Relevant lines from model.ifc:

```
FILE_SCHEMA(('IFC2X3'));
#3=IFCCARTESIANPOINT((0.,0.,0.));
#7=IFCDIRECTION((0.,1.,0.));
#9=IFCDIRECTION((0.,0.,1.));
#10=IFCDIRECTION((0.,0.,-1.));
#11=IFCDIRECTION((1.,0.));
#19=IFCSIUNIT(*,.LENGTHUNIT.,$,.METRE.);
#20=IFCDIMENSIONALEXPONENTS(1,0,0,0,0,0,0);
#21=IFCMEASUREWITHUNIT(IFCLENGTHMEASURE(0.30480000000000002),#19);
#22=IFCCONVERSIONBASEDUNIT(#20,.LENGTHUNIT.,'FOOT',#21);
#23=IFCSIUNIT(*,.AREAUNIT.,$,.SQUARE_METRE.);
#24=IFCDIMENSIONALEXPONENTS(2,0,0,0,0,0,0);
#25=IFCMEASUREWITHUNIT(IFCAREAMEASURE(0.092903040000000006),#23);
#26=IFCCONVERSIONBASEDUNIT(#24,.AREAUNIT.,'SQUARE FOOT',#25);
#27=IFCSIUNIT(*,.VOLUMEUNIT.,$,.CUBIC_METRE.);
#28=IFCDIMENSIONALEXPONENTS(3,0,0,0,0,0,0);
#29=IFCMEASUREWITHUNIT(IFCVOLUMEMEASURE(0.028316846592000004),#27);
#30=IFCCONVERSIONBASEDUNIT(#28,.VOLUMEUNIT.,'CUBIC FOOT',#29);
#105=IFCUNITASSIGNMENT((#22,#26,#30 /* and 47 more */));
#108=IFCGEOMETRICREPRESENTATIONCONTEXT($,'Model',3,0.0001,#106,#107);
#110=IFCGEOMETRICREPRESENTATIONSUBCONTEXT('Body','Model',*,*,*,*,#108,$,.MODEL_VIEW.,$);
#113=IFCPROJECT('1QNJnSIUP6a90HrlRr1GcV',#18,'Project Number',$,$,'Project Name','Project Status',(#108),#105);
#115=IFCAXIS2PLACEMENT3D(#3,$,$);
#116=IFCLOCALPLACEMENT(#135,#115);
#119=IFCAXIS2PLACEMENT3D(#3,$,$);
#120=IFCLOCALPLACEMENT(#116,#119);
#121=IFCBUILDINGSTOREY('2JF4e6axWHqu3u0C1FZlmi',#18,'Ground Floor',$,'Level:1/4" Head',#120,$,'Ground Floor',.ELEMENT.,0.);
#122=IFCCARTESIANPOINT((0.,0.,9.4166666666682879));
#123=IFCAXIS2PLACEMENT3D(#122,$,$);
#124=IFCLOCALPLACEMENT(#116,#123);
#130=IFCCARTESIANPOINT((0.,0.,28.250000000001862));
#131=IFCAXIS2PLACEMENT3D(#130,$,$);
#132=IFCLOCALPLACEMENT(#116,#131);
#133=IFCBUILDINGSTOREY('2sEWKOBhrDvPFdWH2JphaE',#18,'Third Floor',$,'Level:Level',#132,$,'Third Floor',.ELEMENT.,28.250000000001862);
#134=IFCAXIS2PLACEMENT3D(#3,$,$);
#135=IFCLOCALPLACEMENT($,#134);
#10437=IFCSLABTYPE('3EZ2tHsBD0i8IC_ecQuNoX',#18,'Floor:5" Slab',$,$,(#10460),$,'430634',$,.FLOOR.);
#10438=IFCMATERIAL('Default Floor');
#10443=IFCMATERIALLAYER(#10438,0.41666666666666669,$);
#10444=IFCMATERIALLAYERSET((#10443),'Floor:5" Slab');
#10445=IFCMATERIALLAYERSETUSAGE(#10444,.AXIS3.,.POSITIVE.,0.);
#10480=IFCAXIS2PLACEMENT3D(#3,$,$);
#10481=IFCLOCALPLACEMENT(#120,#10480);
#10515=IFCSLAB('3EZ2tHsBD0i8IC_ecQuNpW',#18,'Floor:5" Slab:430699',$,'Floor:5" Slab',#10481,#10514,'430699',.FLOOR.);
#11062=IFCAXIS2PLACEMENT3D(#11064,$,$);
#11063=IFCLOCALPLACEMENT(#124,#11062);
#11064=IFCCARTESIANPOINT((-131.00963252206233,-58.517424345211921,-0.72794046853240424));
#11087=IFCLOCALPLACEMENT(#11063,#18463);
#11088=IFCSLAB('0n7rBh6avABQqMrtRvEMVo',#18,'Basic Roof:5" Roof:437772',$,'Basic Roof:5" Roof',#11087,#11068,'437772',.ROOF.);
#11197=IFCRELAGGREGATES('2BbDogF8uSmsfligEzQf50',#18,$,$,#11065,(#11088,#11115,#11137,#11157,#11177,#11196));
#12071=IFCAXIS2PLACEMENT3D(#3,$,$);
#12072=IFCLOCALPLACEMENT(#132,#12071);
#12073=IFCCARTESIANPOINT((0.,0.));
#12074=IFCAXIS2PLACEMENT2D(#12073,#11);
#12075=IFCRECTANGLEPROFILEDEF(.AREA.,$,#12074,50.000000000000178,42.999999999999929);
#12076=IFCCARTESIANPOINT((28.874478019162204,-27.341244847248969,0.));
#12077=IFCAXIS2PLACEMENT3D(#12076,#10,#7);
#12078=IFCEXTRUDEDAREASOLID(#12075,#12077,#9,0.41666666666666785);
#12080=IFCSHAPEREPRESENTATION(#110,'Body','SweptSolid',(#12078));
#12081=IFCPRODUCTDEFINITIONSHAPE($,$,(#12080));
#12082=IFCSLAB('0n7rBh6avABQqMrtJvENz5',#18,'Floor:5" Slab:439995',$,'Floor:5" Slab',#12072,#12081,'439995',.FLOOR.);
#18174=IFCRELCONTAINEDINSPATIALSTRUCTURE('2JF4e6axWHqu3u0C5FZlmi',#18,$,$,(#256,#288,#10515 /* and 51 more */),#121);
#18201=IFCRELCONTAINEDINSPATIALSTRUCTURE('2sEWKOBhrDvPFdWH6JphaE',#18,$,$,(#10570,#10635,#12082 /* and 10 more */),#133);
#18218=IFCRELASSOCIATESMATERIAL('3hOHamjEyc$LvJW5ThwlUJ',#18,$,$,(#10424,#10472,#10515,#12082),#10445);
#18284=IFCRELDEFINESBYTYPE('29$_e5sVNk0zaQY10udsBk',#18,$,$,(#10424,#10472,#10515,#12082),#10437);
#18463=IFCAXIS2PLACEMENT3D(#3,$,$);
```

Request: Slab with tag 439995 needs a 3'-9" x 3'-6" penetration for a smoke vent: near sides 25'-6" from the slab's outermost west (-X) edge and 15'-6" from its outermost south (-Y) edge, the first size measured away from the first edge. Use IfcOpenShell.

```python
import numpy as np
import ifcopenshell
import ifcopenshell.api.feature
import ifcopenshell.api.geometry
import ifcopenshell.api.root
import ifcopenshell.geom
import ifcopenshell.util.placement
import ifcopenshell.util.representation
import ifcopenshell.util.shape
import ifcopenshell.util.unit

model = ifcopenshell.open("model.ifc")
unit_scale = ifcopenshell.util.unit.calculate_unit_scale(model)
settings = ifcopenshell.geom.settings()


def volume(element):
    """Net volume in cubic metres, openings subtracted."""
    shape = ifcopenshell.geom.create_shape(settings, element)
    return ifcopenshell.util.shape.get_volume(shape.geometry)


slab = model.by_guid("0n7rBh6avABQqMrtJvENz5")
before = volume(slab)

# Extent in the slab's own axes, in metres. The edges named are its -X and -Y sides.
slab_shape = ifcopenshell.geom.create_shape(settings, slab)
vertices = ifcopenshell.util.shape.get_vertices(slab_shape.geometry)
x_min, y_min, bottom = vertices.min(axis=0)
top = vertices[:, 2].max()

opening = ifcopenshell.api.root.create_entity(model, ifc_class="IfcOpeningElement", name="Smoke vent opening")
context = ifcopenshell.util.representation.get_context(model, "Model", "Body", "MODEL_VIEW")
width, depth = 1.143, 1.0668
outline = [(0.0, 0.0), (width, 0.0), (width, depth), (0.0, depth), (0.0, 0.0)]
# Overshoot both faces by 50 mm so the cut is clean.
shape = ifcopenshell.api.geometry.add_slab_representation(
    model, context=context, depth=top - bottom + 0.1, polyline=outline
)
ifcopenshell.api.geometry.assign_representation(model, product=opening, representation=shape)

matrix = ifcopenshell.util.placement.get_local_placement(slab.ObjectPlacement)
matrix[:, 3] = matrix @ np.append(np.array([x_min + 7.7724, y_min + 4.7244, bottom - 0.05]) / unit_scale, 1.0)
ifcopenshell.api.geometry.edit_object_placement(model, product=opening, matrix=matrix, is_si=False)
ifcopenshell.api.feature.add_feature(model, feature=opening, element=slab)

after = volume(slab)

print(f"slab volume {before:.3f} -> {after:.3f} m3")

model.write("model_rev.ifc")
```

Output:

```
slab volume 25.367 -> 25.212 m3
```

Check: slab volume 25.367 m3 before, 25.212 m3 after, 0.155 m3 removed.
